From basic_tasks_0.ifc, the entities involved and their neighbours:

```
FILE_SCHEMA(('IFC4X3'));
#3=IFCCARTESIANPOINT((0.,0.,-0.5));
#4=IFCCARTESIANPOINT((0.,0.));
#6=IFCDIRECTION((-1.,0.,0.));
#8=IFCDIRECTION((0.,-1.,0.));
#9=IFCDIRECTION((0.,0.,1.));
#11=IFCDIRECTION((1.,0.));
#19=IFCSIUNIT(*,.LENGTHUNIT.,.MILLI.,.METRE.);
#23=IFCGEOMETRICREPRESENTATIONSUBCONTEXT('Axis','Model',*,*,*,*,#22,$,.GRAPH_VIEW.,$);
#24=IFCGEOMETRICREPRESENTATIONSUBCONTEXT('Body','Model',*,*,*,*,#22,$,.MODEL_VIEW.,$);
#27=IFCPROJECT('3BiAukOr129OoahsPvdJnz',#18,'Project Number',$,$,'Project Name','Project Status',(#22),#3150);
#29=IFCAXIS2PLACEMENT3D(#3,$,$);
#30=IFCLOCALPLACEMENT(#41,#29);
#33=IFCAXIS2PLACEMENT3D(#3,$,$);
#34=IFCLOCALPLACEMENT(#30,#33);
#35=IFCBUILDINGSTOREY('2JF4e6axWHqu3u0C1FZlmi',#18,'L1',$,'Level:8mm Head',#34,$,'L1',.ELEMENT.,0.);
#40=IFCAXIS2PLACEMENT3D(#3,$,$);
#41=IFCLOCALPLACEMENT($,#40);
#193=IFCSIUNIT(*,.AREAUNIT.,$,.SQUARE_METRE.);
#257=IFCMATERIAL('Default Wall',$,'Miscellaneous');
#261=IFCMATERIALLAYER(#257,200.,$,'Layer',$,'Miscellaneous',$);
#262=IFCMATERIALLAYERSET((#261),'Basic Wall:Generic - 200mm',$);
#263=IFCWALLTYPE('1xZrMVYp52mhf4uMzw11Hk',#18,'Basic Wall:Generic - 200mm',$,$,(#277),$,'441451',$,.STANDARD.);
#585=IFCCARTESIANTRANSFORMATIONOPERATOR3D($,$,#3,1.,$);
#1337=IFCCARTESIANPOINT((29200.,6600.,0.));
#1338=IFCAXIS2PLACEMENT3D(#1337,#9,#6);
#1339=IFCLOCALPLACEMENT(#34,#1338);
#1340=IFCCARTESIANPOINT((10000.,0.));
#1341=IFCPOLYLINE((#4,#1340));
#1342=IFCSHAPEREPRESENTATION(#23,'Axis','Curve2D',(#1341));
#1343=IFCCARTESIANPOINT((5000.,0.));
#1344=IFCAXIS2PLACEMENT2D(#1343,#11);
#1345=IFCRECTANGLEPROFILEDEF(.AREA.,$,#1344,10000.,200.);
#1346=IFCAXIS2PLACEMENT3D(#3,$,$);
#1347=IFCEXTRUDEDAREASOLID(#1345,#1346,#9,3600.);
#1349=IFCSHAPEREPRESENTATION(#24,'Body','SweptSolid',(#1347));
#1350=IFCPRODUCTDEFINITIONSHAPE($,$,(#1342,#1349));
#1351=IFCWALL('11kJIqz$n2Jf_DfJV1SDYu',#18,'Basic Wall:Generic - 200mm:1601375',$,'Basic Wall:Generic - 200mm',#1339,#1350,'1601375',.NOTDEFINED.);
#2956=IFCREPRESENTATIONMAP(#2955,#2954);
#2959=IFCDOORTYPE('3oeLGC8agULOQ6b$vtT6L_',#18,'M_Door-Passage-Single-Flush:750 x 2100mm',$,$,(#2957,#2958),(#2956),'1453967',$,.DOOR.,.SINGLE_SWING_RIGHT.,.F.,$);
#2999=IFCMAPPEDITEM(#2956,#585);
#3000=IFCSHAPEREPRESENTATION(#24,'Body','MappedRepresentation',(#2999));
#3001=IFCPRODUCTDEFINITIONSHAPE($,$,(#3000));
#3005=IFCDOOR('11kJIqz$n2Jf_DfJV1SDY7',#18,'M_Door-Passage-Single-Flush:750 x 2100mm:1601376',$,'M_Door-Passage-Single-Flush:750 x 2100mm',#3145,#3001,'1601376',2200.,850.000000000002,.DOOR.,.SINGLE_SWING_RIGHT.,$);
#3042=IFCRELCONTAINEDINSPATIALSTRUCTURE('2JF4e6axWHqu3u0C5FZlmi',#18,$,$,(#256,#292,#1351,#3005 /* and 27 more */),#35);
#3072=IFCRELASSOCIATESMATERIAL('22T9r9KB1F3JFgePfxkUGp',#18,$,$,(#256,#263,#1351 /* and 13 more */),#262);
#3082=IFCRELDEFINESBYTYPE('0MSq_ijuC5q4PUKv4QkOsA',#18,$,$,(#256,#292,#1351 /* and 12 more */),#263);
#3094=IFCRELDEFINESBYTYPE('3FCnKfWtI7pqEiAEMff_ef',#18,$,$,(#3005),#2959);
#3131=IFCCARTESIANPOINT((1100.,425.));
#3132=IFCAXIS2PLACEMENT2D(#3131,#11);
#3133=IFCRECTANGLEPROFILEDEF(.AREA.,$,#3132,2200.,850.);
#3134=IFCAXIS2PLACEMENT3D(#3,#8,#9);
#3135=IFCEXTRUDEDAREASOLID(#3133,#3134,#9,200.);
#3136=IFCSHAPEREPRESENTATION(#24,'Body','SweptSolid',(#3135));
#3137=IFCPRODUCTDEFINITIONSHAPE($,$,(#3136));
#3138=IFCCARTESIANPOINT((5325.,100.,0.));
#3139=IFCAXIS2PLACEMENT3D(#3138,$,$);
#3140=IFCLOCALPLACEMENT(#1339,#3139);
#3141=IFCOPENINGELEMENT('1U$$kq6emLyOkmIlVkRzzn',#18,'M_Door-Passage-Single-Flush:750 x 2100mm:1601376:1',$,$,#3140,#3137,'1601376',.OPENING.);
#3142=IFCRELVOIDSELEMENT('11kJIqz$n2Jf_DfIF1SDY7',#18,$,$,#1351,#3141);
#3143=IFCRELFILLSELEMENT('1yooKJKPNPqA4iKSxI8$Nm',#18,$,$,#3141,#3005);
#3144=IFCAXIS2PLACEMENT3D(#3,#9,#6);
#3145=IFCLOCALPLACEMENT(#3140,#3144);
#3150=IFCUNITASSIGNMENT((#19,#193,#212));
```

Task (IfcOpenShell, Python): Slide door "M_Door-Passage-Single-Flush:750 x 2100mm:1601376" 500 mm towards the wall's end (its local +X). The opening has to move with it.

```python
import ifcopenshell
import ifcopenshell.api.geometry
import ifcopenshell.util.placement

model = ifcopenshell.open("basic_tasks_0.ifc")

door = model.by_guid("11kJIqz$n2Jf_DfJV1SDY7")
opening = door.FillsVoids[0].RelatingOpeningElement
wall = opening.VoidsElements[0].RelatingBuildingElement

wall_matrix = ifcopenshell.util.placement.get_local_placement(wall.ObjectPlacement)
shift = wall_matrix[:3, 0] * 500.0
before = ifcopenshell.util.placement.get_local_placement(door.ObjectPlacement)[:3, 3].copy()

# The door is placed relative to its opening, so it follows when the opening moves.
matrix = ifcopenshell.util.placement.get_local_placement(opening.ObjectPlacement)
matrix[:3, 3] += shift
ifcopenshell.api.geometry.edit_object_placement(
    model, product=opening, matrix=matrix, is_si=False, should_transform_children=True
)

after = ifcopenshell.util.placement.get_local_placement(door.ObjectPlacement)[:3, 3]
print("door moved by", (after - before).round(3) + 0.0)

model.write("basic_tasks_0_edited.ifc")
```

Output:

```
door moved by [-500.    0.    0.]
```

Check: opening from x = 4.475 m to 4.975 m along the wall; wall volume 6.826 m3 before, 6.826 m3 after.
